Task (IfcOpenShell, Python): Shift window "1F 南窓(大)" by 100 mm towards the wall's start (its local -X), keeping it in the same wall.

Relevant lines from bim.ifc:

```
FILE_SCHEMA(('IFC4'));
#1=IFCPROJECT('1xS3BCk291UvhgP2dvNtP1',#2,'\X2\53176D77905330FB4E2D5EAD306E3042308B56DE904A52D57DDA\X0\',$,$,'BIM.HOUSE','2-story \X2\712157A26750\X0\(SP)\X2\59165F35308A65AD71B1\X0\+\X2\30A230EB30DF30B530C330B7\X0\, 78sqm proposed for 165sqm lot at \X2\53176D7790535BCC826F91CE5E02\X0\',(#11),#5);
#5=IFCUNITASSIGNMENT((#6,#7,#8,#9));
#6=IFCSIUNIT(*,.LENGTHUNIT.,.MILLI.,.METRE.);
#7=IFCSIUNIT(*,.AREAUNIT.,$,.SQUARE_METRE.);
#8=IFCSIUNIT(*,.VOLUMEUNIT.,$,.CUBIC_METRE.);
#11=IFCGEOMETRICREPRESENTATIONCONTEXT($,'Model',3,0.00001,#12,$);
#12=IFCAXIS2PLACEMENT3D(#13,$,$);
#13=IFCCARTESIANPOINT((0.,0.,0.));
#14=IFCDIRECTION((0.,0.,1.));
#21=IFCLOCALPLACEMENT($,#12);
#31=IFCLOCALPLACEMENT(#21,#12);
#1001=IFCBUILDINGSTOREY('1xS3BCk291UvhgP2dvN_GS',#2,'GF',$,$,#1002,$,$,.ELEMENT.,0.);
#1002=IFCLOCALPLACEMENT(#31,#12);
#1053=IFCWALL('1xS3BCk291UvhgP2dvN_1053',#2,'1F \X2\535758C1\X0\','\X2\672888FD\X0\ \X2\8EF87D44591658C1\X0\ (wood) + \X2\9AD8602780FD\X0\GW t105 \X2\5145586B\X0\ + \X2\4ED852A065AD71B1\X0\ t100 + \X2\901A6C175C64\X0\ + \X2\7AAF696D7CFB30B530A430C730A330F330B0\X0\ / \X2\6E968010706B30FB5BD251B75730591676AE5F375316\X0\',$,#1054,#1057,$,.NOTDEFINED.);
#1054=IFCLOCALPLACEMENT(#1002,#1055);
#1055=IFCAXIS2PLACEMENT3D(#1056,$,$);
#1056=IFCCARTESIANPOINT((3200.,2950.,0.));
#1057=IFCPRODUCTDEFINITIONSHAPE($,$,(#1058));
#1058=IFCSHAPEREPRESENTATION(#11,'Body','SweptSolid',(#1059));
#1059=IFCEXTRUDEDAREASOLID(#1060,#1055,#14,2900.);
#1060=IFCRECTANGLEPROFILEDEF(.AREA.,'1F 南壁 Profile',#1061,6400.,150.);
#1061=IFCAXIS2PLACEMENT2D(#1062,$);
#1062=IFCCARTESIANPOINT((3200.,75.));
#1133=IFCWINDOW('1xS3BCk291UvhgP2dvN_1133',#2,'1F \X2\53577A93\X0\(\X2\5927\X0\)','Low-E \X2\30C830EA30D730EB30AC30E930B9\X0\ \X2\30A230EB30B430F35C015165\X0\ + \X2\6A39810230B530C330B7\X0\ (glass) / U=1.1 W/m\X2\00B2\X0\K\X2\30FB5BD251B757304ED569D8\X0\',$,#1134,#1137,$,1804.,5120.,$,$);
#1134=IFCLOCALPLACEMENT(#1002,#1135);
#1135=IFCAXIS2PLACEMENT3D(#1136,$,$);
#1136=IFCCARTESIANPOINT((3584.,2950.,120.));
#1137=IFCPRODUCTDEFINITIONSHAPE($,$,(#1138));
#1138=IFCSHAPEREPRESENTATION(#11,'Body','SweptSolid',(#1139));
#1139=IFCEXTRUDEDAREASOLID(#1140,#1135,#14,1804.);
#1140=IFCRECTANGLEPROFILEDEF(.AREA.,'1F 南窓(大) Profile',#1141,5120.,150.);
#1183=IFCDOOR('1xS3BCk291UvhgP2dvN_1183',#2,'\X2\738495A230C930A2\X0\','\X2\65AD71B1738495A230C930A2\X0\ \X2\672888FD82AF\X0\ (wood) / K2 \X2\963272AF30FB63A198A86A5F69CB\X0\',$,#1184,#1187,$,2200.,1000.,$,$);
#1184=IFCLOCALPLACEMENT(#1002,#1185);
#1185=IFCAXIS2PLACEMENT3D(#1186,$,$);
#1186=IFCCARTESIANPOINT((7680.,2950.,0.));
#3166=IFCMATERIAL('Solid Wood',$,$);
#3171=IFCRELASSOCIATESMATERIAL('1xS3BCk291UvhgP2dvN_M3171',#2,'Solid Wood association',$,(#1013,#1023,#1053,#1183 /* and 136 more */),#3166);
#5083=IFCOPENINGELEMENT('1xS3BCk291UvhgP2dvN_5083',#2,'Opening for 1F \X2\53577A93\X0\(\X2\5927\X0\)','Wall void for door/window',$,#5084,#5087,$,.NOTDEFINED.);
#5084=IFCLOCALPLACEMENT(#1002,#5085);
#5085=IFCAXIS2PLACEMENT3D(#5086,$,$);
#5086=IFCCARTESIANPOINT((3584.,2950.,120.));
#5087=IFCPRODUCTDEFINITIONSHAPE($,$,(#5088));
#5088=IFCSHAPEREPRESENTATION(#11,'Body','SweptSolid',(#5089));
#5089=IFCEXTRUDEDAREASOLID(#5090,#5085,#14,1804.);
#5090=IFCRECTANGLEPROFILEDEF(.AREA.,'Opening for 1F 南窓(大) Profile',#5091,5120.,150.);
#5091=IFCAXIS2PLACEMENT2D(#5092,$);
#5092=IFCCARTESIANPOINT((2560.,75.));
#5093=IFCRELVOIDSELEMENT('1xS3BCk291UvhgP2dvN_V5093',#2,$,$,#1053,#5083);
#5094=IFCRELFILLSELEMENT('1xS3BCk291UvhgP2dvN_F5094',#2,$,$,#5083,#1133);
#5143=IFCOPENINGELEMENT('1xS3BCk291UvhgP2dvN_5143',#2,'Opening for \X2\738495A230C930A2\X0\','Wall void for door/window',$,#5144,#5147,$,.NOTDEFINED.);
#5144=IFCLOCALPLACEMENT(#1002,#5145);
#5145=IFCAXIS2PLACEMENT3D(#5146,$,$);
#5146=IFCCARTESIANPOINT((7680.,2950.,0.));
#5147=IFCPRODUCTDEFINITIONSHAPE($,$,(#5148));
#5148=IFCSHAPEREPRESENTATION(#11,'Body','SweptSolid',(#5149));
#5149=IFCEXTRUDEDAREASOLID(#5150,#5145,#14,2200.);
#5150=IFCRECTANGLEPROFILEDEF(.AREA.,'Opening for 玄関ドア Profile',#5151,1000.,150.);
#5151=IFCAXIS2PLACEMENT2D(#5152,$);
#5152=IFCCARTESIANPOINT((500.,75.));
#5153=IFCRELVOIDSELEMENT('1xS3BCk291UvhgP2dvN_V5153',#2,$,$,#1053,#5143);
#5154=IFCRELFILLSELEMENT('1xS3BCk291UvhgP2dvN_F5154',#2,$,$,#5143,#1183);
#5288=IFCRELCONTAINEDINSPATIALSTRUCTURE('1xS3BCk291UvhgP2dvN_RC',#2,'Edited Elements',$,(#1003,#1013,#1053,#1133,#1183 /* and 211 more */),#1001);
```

```python
import ifcopenshell
import ifcopenshell.api.geometry
import ifcopenshell.util.placement

model = ifcopenshell.open("bim.ifc")

window = model.by_guid("1xS3BCk291UvhgP2dvN_1133")
opening = window.FillsVoids[0].RelatingOpeningElement
wall = opening.VoidsElements[0].RelatingBuildingElement

wall_matrix = ifcopenshell.util.placement.get_local_placement(wall.ObjectPlacement)
shift = wall_matrix[:3, 0] * -100.0
before = ifcopenshell.util.placement.get_local_placement(window.ObjectPlacement)[:3, 3].copy()

# The window is not placed relative to its opening, so move both.
for product in (opening, window):
    matrix = ifcopenshell.util.placement.get_local_placement(product.ObjectPlacement)
    matrix[:3, 3] += shift
    ifcopenshell.api.geometry.edit_object_placement(model, product=product, matrix=matrix, is_si=False)

after = ifcopenshell.util.placement.get_local_placement(window.ObjectPlacement)[:3, 3]
print("window moved by", (after - before).round(3) + 0.0)

model.write("bim_updated.ifc")
```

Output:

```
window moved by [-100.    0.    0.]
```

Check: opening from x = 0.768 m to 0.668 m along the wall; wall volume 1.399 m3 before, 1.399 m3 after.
